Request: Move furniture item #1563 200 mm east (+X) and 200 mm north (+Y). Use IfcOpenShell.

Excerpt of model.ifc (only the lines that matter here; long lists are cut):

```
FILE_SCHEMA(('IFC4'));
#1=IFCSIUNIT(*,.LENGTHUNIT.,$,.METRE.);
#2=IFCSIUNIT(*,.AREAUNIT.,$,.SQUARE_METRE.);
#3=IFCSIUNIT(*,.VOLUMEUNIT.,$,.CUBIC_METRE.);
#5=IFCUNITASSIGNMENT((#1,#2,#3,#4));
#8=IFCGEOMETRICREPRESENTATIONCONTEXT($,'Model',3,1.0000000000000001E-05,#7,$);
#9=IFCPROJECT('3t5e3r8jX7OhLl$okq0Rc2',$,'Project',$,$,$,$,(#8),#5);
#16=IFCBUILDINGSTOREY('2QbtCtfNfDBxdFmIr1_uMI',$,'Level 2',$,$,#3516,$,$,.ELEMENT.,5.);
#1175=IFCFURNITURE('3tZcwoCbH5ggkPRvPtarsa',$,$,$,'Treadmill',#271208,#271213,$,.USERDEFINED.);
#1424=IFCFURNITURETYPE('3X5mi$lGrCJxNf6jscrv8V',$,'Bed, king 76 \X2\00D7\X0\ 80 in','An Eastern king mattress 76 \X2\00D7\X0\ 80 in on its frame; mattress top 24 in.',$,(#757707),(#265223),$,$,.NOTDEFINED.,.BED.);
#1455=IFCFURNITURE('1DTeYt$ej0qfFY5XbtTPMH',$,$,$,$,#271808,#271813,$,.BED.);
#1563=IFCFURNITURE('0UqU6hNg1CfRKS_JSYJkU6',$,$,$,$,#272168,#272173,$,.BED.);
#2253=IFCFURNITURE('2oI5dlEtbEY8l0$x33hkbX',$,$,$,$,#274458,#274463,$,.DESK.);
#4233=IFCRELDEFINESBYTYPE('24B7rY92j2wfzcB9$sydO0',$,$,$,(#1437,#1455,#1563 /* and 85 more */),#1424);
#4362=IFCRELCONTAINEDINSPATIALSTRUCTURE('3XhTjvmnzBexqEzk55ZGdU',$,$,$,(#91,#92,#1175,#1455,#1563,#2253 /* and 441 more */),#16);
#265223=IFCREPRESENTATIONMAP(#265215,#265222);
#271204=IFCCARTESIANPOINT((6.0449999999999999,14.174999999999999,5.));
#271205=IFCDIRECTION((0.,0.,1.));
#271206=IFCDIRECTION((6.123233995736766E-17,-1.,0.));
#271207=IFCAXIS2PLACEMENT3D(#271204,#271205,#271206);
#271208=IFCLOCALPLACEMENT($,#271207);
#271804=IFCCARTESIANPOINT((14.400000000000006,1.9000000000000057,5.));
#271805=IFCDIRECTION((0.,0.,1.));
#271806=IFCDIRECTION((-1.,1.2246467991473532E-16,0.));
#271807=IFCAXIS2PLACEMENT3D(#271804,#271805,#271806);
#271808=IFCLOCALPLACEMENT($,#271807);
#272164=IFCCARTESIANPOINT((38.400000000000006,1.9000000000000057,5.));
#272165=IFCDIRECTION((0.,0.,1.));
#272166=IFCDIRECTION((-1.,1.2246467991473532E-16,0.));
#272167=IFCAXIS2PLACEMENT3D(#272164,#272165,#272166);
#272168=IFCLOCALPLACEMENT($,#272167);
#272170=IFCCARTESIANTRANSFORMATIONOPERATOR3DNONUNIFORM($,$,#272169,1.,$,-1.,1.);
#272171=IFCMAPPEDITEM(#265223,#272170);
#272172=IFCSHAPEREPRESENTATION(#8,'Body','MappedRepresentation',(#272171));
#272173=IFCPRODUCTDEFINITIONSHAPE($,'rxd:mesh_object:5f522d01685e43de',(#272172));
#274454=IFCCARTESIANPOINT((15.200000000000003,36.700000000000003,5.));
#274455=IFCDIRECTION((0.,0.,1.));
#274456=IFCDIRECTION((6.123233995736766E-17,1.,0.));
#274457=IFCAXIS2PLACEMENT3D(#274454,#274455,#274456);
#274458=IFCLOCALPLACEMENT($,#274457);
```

```python
import ifcopenshell
import ifcopenshell.api.geometry
import ifcopenshell.util.placement
import ifcopenshell.util.unit

model = ifcopenshell.open("model.ifc")
unit_scale = ifcopenshell.util.unit.calculate_unit_scale(model)

item = model.by_id(1563)
matrix = ifcopenshell.util.placement.get_local_placement(item.ObjectPlacement)
matrix[0, 3] += 0.2 / unit_scale
matrix[1, 3] += 0.2 / unit_scale
ifcopenshell.api.geometry.edit_object_placement(model, product=item, matrix=matrix, is_si=False)

print(ifcopenshell.util.placement.get_local_placement(item.ObjectPlacement).round(3) + 0.0)

model.write("model_v2.ifc")
```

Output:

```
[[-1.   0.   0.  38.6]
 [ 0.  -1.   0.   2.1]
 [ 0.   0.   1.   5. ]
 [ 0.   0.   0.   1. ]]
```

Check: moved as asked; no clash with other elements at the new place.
